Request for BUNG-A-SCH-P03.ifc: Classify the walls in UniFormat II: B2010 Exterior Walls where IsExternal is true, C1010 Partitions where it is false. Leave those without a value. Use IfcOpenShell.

First a look at what the model holds.

```python
import ifcopenshell
import ifcopenshell.util.element

model = ifcopenshell.open("BUNG-A-SCH-P03.ifc")
print(model.schema)
print("classifications:", [c.Name for c in model.by_type("IfcClassification")])
values = [ifcopenshell.util.element.get_pset(e, "Pset_WallCommon", "IsExternal") for e in model.by_type("IfcWall")]
for value in (True, False, None):
    print("IsExternal", value, values.count(value))
```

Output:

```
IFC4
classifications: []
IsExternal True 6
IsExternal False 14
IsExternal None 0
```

```python
import ifcopenshell
import ifcopenshell.api.classification
import ifcopenshell.util.element

model = ifcopenshell.open("BUNG-A-SCH-P03.ifc")

system = ifcopenshell.api.classification.add_classification(model, classification="UniFormat II")

walls = model.by_type("IfcWall")
external = {e: ifcopenshell.util.element.get_pset(e, "Pset_WallCommon", "IsExternal") for e in walls}
for flag, code, name in ((True, "B2010", "Exterior Walls"), (False, "C1010", "Partitions")):
    products = [e for e in walls if external[e] is flag]
    ifcopenshell.api.classification.add_reference(
        model, products=products, classification=system, identification=code, name=name
    )
    print(code, len(products))

model.write("BUNG-A-SCH-P03_v2.ifc")
```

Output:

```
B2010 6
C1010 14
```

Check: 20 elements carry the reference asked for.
